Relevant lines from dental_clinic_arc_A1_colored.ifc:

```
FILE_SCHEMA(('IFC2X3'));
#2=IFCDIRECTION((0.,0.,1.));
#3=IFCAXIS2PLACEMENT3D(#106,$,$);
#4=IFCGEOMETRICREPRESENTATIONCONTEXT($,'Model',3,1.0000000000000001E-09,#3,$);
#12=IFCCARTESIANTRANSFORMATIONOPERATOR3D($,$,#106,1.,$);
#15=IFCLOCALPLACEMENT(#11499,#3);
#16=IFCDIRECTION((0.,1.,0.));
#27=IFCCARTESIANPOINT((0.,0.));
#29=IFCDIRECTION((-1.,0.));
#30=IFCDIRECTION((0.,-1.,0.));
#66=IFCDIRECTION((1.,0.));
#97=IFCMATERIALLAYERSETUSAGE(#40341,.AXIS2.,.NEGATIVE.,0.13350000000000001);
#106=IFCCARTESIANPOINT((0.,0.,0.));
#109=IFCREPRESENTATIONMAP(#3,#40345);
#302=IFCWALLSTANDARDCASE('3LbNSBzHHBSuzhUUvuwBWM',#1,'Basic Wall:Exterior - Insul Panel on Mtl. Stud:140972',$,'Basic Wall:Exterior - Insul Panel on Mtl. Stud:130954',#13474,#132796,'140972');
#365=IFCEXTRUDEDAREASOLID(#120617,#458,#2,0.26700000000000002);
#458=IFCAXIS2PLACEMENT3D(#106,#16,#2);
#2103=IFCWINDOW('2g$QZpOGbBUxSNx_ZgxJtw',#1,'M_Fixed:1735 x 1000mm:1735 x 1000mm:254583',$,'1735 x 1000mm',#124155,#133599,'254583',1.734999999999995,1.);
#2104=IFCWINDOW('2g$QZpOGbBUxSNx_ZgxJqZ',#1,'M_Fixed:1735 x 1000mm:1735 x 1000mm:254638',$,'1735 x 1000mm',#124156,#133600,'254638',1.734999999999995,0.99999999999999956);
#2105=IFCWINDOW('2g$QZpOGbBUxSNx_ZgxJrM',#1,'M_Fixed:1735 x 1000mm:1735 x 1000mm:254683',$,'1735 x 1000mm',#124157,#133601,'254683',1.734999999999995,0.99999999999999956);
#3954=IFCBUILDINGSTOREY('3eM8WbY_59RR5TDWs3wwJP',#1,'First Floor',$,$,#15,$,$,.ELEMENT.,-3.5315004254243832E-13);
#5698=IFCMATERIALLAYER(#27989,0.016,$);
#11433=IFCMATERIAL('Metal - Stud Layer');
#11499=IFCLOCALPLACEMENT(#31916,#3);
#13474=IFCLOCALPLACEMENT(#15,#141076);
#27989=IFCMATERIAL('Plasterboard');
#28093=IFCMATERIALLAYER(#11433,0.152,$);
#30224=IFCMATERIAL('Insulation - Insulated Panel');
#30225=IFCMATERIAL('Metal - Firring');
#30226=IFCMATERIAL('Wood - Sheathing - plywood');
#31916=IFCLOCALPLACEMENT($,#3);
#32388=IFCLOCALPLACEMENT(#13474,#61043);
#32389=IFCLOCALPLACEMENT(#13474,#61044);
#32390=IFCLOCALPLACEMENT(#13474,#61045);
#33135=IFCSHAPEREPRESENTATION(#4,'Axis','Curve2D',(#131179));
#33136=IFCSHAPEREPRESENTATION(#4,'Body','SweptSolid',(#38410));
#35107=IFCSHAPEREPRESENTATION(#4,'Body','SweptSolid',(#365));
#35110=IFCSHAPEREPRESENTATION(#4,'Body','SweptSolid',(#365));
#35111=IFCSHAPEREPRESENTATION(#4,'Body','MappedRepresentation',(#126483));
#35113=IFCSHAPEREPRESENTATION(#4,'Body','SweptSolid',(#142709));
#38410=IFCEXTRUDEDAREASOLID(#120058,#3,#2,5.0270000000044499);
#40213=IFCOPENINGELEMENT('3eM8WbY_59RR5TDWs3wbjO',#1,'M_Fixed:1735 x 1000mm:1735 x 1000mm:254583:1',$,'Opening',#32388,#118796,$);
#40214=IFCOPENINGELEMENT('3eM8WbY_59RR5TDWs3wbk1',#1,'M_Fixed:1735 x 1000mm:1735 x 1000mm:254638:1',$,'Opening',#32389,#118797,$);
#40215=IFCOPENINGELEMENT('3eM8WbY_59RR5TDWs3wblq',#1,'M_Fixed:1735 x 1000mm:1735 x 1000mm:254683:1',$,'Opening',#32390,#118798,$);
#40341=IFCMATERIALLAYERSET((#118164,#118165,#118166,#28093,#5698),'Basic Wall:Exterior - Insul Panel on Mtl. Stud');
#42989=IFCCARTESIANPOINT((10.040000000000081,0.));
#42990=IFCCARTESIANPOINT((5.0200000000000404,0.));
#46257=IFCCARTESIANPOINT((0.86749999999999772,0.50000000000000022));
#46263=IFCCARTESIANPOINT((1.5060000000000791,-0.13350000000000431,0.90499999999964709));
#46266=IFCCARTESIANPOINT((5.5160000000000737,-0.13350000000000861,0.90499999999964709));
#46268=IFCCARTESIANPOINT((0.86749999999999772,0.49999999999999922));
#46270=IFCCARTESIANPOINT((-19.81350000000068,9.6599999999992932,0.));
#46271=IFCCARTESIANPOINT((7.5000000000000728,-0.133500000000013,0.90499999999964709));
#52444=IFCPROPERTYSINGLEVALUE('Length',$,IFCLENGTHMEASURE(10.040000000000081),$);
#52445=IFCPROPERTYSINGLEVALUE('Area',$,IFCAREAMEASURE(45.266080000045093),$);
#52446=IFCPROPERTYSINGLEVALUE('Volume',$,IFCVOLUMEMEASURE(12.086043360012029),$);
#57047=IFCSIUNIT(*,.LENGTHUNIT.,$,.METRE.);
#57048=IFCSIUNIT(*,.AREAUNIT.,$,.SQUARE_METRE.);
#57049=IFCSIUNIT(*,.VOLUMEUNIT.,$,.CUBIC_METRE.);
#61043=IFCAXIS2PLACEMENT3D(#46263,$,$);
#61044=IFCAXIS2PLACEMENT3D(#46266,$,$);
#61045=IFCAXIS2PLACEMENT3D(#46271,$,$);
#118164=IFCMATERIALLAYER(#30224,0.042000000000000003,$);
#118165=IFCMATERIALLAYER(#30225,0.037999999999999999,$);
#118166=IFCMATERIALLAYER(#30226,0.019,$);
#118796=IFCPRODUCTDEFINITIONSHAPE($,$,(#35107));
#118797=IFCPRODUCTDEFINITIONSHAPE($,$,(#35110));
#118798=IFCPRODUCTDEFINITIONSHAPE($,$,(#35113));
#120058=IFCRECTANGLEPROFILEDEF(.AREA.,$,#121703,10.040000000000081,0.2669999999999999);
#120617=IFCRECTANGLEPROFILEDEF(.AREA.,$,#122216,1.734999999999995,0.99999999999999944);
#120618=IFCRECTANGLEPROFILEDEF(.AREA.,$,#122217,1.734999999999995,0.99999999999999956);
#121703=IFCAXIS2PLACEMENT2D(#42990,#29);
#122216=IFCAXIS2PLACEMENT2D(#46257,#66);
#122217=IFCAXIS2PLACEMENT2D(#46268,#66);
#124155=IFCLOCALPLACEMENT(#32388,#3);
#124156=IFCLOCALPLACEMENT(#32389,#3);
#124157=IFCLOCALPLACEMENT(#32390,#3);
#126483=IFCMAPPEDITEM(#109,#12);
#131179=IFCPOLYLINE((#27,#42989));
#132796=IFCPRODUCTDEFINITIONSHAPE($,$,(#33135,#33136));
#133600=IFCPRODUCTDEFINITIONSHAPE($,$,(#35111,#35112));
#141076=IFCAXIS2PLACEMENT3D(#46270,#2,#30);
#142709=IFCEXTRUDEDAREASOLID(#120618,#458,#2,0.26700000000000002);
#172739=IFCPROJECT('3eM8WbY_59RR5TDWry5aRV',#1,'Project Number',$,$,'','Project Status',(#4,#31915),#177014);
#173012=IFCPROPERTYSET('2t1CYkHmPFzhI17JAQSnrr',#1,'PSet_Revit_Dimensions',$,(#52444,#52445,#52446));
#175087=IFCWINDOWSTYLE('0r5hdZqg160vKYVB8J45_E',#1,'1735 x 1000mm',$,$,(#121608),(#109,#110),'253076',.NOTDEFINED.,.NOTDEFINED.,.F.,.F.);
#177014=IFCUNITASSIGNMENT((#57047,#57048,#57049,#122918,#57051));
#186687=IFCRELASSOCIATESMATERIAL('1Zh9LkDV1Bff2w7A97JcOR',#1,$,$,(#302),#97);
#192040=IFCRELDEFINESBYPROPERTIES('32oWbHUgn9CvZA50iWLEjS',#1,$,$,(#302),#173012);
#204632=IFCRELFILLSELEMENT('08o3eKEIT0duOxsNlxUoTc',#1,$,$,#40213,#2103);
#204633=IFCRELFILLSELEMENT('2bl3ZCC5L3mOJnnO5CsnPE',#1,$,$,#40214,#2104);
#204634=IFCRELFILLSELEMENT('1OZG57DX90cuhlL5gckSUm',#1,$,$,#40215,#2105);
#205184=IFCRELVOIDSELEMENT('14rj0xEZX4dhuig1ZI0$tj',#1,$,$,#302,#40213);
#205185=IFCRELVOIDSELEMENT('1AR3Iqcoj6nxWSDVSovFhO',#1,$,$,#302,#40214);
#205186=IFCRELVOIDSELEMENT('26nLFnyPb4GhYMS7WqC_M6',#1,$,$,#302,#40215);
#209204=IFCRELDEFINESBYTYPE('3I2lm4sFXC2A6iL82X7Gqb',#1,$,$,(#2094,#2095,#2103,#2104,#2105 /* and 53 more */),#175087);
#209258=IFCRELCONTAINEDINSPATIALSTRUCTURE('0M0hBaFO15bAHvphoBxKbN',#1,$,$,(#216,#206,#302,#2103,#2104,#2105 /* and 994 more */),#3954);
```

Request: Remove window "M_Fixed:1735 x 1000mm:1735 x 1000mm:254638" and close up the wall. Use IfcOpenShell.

```python
import ifcopenshell
import ifcopenshell.api.feature
import ifcopenshell.api.pset
import ifcopenshell.api.root
import ifcopenshell.geom
import ifcopenshell.util.element
import ifcopenshell.util.shape
import ifcopenshell.util.unit

model = ifcopenshell.open("dental_clinic_arc_A1_colored.ifc")
area_scale = ifcopenshell.util.unit.calculate_unit_scale(model, "AREAUNIT")
volume_scale = ifcopenshell.util.unit.calculate_unit_scale(model, "VOLUMEUNIT")
settings = ifcopenshell.geom.settings()


def volume(element):
    """Net volume in cubic metres, openings subtracted."""
    shape = ifcopenshell.geom.create_shape(settings, element)
    return ifcopenshell.util.shape.get_volume(shape.geometry)


window = model.by_id(2104)
opening = window.FillsVoids[0].RelatingOpeningElement
wall = opening.VoidsElements[0].RelatingBuildingElement
before = volume(wall)

ifcopenshell.api.root.remove_product(model, product=window)
ifcopenshell.api.feature.remove_feature(model, feature=opening)

after = volume(wall)
thickness = 0.267  # wall thickness in metres

# Update the wall's stored quantities.
pset = model.by_id(ifcopenshell.util.element.get_pset(wall, "PSet_Revit_Dimensions", should_inherit=False)["id"])
ifcopenshell.api.pset.edit_pset(model, pset=pset, properties={
    "Area": model.create_entity("IfcAreaMeasure", after / thickness / area_scale),
    "Volume": model.create_entity("IfcVolumeMeasure", after / volume_scale),
})

print(f"wall volume {before:.3f} -> {after:.3f} m3")

model.write("dental_clinic_arc_A1_colored_edited.ifc")
```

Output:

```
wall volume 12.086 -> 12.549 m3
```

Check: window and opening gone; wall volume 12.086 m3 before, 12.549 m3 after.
